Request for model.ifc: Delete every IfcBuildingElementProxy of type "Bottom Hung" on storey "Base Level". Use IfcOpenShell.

First a look at what the model holds.

```python
import ifcopenshell
import ifcopenshell.util.element

model = ifcopenshell.open("model.ifc")
print(model.schema)
storey = next(s for s in model.by_type("IfcBuildingStorey") if s.Name == "Base Level")
proxies = [e for e in ifcopenshell.util.element.get_decomposition(storey) if e.is_a("IfcBuildingElementProxy")]
seen = {}
for e in proxies:
    element_type = ifcopenshell.util.element.get_type(e)
    name = element_type.Name if element_type not in (None, e) else None
    seen[name] = seen.get(name, 0) + 1
for name, count in sorted(seen.items(), key=str):
    print(count, "x", name)
```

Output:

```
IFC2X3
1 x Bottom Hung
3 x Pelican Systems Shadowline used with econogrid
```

```python
import ifcopenshell
import ifcopenshell.api.root
import ifcopenshell.util.element

model = ifcopenshell.open("model.ifc")

storey = next(s for s in model.by_type("IfcBuildingStorey") if s.Name == "Base Level")
proxies = [e for e in ifcopenshell.util.element.get_decomposition(storey) if e.is_a("IfcBuildingElementProxy")]
targets = [e for e in proxies if (t := ifcopenshell.util.element.get_type(e)) not in (None, e) and t.Name == "Bottom Hung"]

for e in targets:
    ifcopenshell.api.root.remove_product(model, product=e)
print(len(targets), "removed")

model.write("model_v2.ifc")
```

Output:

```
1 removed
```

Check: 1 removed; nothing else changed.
